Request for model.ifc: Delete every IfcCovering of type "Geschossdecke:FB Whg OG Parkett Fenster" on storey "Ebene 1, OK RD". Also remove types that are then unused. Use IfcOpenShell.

First a look at what the model holds.

```python
import ifcopenshell
import ifcopenshell.util.element

model = ifcopenshell.open("model.ifc")
print(model.schema)
storey = next(s for s in model.by_type("IfcBuildingStorey") if s.Name == "Ebene 1, OK RD")
coverings = [e for e in ifcopenshell.util.element.get_decomposition(storey) if e.is_a("IfcCovering")]
seen = {}
for e in coverings:
    element_type = ifcopenshell.util.element.get_type(e)
    name = element_type.Name if element_type not in (None, e) else None
    seen[name] = seen.get(name, 0) + 1
for name, count in sorted(seen.items(), key=str):
    print(count, "x", name)
```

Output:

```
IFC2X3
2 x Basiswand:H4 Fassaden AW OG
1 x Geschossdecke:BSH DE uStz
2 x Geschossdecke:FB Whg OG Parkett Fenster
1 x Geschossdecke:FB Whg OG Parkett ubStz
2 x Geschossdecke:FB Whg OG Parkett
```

```python
import ifcopenshell
import ifcopenshell.api.root
import ifcopenshell.util.element

model = ifcopenshell.open("model.ifc")

storey = next(s for s in model.by_type("IfcBuildingStorey") if s.Name == "Ebene 1, OK RD")
coverings = [e for e in ifcopenshell.util.element.get_decomposition(storey) if e.is_a("IfcCovering")]
targets = [e for e in coverings if (t := ifcopenshell.util.element.get_type(e)) not in (None, e) and t.Name == "Geschossdecke:FB Whg OG Parkett Fenster"]
types = {ifcopenshell.util.element.get_type(e) for e in targets} - {None, *targets}

for e in targets:
    ifcopenshell.api.root.remove_product(model, product=e)
print(len(targets), "removed")

unused = [t for t in types if not ifcopenshell.util.element.get_types(t)]
for t in unused:
    ifcopenshell.api.root.remove_product(model, product=t)
print(len(unused), "unused types removed")

model.write("model_updated.ifc")
```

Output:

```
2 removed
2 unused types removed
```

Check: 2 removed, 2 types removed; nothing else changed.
